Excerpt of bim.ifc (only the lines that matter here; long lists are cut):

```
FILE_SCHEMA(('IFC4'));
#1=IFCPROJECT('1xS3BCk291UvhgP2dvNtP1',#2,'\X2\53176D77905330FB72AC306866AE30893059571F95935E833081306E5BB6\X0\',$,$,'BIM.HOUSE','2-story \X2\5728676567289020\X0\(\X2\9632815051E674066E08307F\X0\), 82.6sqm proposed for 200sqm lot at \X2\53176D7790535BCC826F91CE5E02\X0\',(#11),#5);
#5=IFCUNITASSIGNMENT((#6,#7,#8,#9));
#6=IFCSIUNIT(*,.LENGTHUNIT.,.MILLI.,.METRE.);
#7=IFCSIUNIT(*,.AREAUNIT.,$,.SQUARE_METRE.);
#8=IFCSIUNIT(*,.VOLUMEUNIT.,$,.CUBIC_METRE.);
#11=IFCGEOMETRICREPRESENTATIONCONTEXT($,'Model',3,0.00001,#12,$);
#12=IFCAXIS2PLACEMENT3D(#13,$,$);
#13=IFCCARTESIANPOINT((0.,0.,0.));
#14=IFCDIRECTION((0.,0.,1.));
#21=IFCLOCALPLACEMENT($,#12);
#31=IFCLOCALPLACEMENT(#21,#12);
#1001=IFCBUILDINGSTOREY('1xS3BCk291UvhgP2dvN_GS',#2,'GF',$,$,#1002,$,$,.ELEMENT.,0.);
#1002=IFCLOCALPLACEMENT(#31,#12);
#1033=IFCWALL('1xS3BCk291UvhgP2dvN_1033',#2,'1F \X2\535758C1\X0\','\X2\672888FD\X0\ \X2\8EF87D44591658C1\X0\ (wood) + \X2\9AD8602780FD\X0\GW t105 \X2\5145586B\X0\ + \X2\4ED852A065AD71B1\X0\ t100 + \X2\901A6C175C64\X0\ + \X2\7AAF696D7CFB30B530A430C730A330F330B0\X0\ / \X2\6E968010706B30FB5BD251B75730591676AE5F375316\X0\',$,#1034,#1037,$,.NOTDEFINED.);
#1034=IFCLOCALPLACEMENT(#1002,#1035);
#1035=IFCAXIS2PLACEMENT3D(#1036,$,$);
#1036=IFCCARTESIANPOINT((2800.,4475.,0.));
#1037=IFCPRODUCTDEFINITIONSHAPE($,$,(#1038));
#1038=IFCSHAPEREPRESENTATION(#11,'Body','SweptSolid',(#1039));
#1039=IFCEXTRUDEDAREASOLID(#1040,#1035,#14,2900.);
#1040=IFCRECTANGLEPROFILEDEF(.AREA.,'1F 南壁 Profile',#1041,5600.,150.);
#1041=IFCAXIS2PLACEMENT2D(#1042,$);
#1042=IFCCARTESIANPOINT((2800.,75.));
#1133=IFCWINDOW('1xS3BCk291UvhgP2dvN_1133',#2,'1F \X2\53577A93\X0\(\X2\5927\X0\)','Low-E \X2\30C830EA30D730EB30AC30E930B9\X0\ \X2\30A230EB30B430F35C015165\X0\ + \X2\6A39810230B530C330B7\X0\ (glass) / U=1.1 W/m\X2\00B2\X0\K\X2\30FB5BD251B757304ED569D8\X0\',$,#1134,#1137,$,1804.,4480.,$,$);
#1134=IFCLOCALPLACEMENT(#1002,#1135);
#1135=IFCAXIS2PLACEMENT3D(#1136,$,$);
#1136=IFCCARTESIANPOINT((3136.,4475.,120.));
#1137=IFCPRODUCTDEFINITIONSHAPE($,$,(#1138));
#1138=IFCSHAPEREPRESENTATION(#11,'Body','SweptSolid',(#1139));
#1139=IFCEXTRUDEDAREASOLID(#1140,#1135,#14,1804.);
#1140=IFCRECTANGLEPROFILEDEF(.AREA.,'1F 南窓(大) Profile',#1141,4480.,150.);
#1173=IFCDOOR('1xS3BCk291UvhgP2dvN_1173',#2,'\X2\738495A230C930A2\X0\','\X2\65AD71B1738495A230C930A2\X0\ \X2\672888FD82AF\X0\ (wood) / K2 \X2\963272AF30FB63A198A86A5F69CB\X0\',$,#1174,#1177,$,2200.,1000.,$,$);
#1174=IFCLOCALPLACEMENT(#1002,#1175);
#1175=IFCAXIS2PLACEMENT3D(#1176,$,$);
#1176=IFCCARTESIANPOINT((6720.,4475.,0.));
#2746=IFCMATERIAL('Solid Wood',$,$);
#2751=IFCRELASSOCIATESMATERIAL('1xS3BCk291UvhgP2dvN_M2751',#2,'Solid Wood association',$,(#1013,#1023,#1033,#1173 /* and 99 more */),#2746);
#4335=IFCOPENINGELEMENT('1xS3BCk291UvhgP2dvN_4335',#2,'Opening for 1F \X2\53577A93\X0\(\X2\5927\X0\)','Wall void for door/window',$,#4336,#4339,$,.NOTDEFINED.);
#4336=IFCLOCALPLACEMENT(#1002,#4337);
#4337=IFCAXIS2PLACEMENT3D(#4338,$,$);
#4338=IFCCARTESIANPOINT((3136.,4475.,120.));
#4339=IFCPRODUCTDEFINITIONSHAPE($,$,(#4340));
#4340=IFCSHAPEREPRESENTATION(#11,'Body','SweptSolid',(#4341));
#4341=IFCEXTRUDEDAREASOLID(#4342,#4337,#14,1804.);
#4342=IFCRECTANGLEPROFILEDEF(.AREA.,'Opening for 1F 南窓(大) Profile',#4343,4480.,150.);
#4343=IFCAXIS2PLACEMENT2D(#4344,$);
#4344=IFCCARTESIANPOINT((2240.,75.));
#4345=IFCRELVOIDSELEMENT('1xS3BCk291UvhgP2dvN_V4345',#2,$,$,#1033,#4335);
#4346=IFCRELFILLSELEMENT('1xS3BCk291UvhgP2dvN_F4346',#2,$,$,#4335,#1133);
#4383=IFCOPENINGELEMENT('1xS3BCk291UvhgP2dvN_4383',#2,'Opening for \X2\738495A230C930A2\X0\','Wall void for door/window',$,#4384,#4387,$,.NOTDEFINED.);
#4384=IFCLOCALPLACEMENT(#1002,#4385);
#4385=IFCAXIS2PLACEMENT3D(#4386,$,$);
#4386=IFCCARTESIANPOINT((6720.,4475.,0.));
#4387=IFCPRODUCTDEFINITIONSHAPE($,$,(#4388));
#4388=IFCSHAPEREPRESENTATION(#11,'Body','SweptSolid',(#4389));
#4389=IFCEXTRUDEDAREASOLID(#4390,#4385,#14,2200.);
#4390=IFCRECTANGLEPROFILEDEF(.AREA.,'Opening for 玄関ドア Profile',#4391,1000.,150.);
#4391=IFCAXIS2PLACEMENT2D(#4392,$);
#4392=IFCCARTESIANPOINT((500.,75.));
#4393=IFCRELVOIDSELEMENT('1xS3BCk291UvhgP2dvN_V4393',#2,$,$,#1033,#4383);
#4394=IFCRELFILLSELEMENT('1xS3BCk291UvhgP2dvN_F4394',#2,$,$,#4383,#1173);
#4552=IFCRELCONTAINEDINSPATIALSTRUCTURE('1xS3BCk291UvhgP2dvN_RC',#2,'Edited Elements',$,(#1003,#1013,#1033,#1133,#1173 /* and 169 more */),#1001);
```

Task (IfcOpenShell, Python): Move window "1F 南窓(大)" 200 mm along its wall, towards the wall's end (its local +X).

```python
import ifcopenshell
import ifcopenshell.api.geometry
import ifcopenshell.util.placement
import ifcopenshell.util.unit

model = ifcopenshell.open("bim.ifc")
unit_scale = ifcopenshell.util.unit.calculate_unit_scale(model)

window = model.by_id(1133)
opening = window.FillsVoids[0].RelatingOpeningElement
wall = opening.VoidsElements[0].RelatingBuildingElement

wall_matrix = ifcopenshell.util.placement.get_local_placement(wall.ObjectPlacement)
shift = wall_matrix[:3, 0] * 0.2 / unit_scale
before = ifcopenshell.util.placement.get_local_placement(window.ObjectPlacement)[:3, 3].copy()

# The window is not placed relative to its opening, so move both.
for product in (opening, window):
    matrix = ifcopenshell.util.placement.get_local_placement(product.ObjectPlacement)
    matrix[:3, 3] += shift
    ifcopenshell.api.geometry.edit_object_placement(model, product=product, matrix=matrix, is_si=False)

after = ifcopenshell.util.placement.get_local_placement(window.ObjectPlacement)[:3, 3]
print("window moved by", (after - before).round(3) + 0.0)

model.write("bim_v2.ifc")
```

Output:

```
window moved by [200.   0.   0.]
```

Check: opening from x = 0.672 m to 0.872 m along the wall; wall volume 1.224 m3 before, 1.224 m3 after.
